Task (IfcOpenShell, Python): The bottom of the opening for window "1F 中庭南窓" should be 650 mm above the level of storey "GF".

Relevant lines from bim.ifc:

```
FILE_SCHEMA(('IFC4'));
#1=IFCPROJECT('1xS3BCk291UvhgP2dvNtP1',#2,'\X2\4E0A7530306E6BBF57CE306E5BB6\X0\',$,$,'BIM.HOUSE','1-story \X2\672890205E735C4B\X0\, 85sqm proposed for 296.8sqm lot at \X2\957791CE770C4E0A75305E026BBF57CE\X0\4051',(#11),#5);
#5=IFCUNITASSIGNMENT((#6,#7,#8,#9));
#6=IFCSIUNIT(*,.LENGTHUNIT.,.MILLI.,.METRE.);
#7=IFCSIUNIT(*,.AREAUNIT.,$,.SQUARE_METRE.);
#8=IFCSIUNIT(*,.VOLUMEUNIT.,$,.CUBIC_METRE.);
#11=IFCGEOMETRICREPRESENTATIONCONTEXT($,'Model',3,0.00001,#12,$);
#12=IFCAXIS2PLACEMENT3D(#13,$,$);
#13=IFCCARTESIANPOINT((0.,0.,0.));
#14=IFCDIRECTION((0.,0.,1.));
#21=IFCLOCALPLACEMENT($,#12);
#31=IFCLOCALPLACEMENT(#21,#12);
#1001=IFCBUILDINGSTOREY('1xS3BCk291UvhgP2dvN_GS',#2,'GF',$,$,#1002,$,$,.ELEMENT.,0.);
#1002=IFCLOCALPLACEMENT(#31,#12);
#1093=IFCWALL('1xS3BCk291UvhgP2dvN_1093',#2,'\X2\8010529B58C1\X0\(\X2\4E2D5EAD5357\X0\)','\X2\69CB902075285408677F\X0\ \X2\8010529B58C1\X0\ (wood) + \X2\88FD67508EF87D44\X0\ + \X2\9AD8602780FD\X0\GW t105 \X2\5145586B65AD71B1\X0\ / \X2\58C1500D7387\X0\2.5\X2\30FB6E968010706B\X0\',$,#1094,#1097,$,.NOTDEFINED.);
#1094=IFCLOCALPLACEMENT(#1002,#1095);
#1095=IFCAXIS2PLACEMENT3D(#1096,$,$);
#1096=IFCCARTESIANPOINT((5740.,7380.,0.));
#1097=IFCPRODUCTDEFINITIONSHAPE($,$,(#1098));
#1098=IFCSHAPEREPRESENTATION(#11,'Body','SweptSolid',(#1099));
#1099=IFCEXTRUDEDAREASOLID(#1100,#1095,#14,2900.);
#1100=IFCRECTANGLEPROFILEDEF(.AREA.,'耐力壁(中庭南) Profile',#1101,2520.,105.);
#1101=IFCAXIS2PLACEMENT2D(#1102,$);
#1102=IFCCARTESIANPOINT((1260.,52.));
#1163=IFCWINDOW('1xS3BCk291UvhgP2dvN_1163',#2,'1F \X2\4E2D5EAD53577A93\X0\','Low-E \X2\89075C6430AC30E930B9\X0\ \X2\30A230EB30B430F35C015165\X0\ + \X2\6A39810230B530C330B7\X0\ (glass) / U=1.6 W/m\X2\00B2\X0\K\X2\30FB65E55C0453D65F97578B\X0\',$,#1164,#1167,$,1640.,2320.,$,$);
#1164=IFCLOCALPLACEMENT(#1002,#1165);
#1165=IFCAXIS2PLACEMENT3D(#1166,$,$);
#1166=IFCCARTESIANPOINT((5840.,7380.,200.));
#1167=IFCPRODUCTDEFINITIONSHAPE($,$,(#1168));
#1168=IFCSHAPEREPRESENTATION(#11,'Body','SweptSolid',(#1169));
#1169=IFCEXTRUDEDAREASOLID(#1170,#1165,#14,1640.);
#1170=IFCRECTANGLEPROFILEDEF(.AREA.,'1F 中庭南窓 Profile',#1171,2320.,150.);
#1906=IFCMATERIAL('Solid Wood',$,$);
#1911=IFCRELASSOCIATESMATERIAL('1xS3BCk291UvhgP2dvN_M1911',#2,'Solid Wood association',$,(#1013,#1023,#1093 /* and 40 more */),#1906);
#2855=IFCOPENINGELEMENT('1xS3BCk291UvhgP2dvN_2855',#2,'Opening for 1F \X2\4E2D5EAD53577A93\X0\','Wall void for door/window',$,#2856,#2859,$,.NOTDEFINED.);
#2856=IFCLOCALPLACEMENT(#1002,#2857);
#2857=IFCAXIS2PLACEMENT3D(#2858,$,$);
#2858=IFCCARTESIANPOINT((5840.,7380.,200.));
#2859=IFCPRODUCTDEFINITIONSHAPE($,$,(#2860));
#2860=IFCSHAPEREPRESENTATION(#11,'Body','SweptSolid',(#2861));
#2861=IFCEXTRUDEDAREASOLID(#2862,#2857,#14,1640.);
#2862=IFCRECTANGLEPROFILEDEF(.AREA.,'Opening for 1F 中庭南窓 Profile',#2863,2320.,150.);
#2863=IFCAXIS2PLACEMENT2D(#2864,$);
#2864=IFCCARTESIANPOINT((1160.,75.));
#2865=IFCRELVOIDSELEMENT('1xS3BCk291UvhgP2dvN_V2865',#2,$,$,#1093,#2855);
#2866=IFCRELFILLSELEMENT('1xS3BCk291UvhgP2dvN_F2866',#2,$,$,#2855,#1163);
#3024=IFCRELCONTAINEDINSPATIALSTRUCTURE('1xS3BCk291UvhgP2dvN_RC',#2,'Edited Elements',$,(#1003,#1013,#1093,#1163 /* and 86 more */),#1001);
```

```python
import numpy as np
import ifcopenshell
import ifcopenshell.api.geometry
import ifcopenshell.geom
import ifcopenshell.util.element
import ifcopenshell.util.placement
import ifcopenshell.util.shape
import ifcopenshell.util.unit

model = ifcopenshell.open("bim.ifc")
unit_scale = ifcopenshell.util.unit.calculate_unit_scale(model)

window = model.by_guid("1xS3BCk291UvhgP2dvN_1163")
opening = window.FillsVoids[0].RelatingOpeningElement
storey = ifcopenshell.util.element.get_container(window, ifc_class="IfcBuildingStorey")
level = ifcopenshell.util.placement.get_local_placement(storey.ObjectPlacement)[2, 3]

# The opening's origin need not be at the sill, so measure its lowest point.
shape = ifcopenshell.geom.create_shape(ifcopenshell.geom.settings(), opening)
bottom = ifcopenshell.util.shape.get_shape_bottom_elevation(shape, shape.geometry) / unit_scale
dz = level + 650.0 - bottom

shift = np.array([0.0, 0.0, dz])
# The window is not placed relative to its opening, so move both.
for product in (opening, window):
    matrix = ifcopenshell.util.placement.get_local_placement(product.ObjectPlacement)
    matrix[:3, 3] += shift
    ifcopenshell.api.geometry.edit_object_placement(model, product=product, matrix=matrix, is_si=False)

print(f"moved by {dz * unit_scale:+.3f} m")

model.write("bim_v2.ifc")
```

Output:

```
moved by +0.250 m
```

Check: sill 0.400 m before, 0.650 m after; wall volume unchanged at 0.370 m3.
